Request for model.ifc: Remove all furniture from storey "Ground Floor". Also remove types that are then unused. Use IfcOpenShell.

First a look at what the model holds.

```python
import ifcopenshell
import ifcopenshell.util.element

model = ifcopenshell.open("model.ifc")
print(model.schema)
storey = next(s for s in model.by_type("IfcBuildingStorey") if s.Name == "Ground Floor")
furniture = [e for e in ifcopenshell.util.element.get_decomposition(storey) if e.is_a("IfcFurnishingElement")]
seen = {}
for e in furniture:
    element_type = ifcopenshell.util.element.get_type(e)
    name = element_type.Name if element_type not in (None, e) else None
    seen[name] = seen.get(name, 0) + 1
for name, count in sorted(seen.items(), key=str):
    print(count, "x", name)
```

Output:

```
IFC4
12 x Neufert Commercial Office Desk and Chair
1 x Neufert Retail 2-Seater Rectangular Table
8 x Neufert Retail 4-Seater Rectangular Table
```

```python
import ifcopenshell
import ifcopenshell.api.root
import ifcopenshell.util.element

model = ifcopenshell.open("model.ifc")

storey = next(s for s in model.by_type("IfcBuildingStorey") if s.Name == "Ground Floor")
furniture = [e for e in ifcopenshell.util.element.get_decomposition(storey) if e.is_a("IfcFurnishingElement")]
types = {ifcopenshell.util.element.get_type(e) for e in furniture} - {None, *furniture}

for e in furniture:
    ifcopenshell.api.root.remove_product(model, product=e)
print(len(furniture), "removed")

unused = [t for t in types if not ifcopenshell.util.element.get_types(t)]
for t in unused:
    ifcopenshell.api.root.remove_product(model, product=t)
print(len(unused), "unused types removed")

model.write("model-out.ifc")
```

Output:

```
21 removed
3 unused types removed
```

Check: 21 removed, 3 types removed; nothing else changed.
